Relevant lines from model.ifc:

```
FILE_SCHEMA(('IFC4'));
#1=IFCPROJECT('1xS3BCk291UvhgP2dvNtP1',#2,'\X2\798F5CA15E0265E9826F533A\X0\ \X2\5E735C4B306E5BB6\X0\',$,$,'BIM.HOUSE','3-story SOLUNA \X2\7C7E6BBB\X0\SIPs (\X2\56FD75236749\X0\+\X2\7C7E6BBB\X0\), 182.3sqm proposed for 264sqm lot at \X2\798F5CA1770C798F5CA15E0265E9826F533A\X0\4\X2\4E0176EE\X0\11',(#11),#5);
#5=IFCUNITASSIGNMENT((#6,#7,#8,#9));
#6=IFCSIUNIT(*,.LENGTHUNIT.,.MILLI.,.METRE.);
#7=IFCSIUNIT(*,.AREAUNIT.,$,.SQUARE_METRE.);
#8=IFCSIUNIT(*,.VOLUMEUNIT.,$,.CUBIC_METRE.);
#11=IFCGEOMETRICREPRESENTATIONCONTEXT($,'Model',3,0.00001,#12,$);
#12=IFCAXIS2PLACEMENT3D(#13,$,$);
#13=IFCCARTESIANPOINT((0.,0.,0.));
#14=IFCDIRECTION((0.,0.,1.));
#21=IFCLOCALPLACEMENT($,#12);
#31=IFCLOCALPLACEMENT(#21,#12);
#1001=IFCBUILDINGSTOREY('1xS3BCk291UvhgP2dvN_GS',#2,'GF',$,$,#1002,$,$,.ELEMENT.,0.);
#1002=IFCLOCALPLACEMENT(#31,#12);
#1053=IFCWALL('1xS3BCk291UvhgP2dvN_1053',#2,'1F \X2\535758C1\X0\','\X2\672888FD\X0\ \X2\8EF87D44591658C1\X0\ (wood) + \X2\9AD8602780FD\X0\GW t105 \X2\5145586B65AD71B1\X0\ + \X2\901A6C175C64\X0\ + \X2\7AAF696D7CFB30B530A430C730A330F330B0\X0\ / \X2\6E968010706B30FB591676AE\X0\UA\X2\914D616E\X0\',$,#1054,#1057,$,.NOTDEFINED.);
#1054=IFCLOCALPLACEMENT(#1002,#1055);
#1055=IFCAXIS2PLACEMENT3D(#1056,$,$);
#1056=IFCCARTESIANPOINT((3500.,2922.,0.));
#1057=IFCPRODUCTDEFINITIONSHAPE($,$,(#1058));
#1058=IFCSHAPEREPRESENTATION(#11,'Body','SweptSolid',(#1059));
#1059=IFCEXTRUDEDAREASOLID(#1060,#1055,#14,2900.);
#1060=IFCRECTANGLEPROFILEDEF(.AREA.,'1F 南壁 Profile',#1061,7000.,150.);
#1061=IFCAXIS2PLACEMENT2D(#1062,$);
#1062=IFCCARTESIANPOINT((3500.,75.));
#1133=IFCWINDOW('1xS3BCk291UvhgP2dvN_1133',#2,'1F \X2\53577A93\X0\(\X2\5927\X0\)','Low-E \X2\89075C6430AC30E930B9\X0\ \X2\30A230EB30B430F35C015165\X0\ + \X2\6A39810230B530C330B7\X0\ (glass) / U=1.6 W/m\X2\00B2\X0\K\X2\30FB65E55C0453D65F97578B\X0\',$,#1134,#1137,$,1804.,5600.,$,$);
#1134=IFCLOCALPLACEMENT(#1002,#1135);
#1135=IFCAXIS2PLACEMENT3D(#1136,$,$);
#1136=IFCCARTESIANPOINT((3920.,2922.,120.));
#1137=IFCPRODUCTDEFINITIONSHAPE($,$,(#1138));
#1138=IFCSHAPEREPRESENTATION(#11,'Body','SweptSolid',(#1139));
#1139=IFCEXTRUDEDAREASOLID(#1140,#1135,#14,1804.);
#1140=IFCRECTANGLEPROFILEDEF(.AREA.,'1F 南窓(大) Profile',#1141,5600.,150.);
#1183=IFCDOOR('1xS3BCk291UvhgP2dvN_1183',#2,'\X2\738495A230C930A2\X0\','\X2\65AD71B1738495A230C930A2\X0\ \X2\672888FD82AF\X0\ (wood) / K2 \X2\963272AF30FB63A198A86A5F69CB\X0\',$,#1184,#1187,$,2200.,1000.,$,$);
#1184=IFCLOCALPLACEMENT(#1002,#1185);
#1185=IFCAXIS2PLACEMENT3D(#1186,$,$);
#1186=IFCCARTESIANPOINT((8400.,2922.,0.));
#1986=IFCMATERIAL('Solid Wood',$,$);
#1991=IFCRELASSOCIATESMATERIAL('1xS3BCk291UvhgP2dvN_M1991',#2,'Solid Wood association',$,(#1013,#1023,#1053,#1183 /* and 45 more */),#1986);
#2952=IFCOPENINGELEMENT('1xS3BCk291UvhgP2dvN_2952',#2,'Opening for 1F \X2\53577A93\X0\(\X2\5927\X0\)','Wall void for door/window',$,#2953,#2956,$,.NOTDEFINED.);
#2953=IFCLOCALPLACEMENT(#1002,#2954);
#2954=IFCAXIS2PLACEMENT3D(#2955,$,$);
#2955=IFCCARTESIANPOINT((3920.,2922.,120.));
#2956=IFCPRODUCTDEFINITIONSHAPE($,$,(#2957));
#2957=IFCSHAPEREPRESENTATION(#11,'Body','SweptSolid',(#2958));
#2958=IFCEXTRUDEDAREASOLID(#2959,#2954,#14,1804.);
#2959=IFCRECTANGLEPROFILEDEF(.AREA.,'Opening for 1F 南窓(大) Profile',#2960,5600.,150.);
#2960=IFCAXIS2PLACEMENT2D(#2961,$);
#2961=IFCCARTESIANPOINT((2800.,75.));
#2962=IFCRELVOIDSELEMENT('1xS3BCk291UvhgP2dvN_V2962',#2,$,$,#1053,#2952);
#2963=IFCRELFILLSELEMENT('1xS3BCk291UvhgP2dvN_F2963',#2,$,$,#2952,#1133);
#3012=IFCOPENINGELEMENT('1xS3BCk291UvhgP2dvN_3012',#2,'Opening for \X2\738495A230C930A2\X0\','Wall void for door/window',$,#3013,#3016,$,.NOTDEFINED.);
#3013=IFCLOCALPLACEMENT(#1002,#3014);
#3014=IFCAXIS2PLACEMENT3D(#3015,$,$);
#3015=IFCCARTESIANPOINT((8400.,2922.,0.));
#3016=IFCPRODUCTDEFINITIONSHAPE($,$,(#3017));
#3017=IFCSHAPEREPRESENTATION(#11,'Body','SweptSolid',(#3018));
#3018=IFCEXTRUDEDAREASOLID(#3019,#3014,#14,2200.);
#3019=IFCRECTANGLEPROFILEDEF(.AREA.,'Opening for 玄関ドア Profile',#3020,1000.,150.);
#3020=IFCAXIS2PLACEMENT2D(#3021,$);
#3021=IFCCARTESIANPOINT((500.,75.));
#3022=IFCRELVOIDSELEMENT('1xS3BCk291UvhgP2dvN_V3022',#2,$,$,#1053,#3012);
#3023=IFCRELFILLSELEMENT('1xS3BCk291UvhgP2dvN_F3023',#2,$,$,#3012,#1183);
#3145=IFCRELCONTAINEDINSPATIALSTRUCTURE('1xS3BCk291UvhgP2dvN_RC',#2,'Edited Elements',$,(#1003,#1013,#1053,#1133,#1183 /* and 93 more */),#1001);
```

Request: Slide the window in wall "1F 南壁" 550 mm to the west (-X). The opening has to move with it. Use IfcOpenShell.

```python
import ifcopenshell
import ifcopenshell.api.geometry
import ifcopenshell.util.placement
import ifcopenshell.util.unit

model = ifcopenshell.open("model.ifc")
unit_scale = ifcopenshell.util.unit.calculate_unit_scale(model)

window = model.by_id(1133)
opening = window.FillsVoids[0].RelatingOpeningElement
wall = opening.VoidsElements[0].RelatingBuildingElement

wall_matrix = ifcopenshell.util.placement.get_local_placement(wall.ObjectPlacement)
shift = wall_matrix[:3, 0] * -0.55 / unit_scale
before = ifcopenshell.util.placement.get_local_placement(window.ObjectPlacement)[:3, 3].copy()

# The window is not placed relative to its opening, so move both.
for product in (opening, window):
    matrix = ifcopenshell.util.placement.get_local_placement(product.ObjectPlacement)
    matrix[:3, 3] += shift
    ifcopenshell.api.geometry.edit_object_placement(model, product=product, matrix=matrix, is_si=False)

after = ifcopenshell.util.placement.get_local_placement(window.ObjectPlacement)[:3, 3]
print("window moved by", (after - before).round(3) + 0.0)

model.write("model_v2.ifc")
```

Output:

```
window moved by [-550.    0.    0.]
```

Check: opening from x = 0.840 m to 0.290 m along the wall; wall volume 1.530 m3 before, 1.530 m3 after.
